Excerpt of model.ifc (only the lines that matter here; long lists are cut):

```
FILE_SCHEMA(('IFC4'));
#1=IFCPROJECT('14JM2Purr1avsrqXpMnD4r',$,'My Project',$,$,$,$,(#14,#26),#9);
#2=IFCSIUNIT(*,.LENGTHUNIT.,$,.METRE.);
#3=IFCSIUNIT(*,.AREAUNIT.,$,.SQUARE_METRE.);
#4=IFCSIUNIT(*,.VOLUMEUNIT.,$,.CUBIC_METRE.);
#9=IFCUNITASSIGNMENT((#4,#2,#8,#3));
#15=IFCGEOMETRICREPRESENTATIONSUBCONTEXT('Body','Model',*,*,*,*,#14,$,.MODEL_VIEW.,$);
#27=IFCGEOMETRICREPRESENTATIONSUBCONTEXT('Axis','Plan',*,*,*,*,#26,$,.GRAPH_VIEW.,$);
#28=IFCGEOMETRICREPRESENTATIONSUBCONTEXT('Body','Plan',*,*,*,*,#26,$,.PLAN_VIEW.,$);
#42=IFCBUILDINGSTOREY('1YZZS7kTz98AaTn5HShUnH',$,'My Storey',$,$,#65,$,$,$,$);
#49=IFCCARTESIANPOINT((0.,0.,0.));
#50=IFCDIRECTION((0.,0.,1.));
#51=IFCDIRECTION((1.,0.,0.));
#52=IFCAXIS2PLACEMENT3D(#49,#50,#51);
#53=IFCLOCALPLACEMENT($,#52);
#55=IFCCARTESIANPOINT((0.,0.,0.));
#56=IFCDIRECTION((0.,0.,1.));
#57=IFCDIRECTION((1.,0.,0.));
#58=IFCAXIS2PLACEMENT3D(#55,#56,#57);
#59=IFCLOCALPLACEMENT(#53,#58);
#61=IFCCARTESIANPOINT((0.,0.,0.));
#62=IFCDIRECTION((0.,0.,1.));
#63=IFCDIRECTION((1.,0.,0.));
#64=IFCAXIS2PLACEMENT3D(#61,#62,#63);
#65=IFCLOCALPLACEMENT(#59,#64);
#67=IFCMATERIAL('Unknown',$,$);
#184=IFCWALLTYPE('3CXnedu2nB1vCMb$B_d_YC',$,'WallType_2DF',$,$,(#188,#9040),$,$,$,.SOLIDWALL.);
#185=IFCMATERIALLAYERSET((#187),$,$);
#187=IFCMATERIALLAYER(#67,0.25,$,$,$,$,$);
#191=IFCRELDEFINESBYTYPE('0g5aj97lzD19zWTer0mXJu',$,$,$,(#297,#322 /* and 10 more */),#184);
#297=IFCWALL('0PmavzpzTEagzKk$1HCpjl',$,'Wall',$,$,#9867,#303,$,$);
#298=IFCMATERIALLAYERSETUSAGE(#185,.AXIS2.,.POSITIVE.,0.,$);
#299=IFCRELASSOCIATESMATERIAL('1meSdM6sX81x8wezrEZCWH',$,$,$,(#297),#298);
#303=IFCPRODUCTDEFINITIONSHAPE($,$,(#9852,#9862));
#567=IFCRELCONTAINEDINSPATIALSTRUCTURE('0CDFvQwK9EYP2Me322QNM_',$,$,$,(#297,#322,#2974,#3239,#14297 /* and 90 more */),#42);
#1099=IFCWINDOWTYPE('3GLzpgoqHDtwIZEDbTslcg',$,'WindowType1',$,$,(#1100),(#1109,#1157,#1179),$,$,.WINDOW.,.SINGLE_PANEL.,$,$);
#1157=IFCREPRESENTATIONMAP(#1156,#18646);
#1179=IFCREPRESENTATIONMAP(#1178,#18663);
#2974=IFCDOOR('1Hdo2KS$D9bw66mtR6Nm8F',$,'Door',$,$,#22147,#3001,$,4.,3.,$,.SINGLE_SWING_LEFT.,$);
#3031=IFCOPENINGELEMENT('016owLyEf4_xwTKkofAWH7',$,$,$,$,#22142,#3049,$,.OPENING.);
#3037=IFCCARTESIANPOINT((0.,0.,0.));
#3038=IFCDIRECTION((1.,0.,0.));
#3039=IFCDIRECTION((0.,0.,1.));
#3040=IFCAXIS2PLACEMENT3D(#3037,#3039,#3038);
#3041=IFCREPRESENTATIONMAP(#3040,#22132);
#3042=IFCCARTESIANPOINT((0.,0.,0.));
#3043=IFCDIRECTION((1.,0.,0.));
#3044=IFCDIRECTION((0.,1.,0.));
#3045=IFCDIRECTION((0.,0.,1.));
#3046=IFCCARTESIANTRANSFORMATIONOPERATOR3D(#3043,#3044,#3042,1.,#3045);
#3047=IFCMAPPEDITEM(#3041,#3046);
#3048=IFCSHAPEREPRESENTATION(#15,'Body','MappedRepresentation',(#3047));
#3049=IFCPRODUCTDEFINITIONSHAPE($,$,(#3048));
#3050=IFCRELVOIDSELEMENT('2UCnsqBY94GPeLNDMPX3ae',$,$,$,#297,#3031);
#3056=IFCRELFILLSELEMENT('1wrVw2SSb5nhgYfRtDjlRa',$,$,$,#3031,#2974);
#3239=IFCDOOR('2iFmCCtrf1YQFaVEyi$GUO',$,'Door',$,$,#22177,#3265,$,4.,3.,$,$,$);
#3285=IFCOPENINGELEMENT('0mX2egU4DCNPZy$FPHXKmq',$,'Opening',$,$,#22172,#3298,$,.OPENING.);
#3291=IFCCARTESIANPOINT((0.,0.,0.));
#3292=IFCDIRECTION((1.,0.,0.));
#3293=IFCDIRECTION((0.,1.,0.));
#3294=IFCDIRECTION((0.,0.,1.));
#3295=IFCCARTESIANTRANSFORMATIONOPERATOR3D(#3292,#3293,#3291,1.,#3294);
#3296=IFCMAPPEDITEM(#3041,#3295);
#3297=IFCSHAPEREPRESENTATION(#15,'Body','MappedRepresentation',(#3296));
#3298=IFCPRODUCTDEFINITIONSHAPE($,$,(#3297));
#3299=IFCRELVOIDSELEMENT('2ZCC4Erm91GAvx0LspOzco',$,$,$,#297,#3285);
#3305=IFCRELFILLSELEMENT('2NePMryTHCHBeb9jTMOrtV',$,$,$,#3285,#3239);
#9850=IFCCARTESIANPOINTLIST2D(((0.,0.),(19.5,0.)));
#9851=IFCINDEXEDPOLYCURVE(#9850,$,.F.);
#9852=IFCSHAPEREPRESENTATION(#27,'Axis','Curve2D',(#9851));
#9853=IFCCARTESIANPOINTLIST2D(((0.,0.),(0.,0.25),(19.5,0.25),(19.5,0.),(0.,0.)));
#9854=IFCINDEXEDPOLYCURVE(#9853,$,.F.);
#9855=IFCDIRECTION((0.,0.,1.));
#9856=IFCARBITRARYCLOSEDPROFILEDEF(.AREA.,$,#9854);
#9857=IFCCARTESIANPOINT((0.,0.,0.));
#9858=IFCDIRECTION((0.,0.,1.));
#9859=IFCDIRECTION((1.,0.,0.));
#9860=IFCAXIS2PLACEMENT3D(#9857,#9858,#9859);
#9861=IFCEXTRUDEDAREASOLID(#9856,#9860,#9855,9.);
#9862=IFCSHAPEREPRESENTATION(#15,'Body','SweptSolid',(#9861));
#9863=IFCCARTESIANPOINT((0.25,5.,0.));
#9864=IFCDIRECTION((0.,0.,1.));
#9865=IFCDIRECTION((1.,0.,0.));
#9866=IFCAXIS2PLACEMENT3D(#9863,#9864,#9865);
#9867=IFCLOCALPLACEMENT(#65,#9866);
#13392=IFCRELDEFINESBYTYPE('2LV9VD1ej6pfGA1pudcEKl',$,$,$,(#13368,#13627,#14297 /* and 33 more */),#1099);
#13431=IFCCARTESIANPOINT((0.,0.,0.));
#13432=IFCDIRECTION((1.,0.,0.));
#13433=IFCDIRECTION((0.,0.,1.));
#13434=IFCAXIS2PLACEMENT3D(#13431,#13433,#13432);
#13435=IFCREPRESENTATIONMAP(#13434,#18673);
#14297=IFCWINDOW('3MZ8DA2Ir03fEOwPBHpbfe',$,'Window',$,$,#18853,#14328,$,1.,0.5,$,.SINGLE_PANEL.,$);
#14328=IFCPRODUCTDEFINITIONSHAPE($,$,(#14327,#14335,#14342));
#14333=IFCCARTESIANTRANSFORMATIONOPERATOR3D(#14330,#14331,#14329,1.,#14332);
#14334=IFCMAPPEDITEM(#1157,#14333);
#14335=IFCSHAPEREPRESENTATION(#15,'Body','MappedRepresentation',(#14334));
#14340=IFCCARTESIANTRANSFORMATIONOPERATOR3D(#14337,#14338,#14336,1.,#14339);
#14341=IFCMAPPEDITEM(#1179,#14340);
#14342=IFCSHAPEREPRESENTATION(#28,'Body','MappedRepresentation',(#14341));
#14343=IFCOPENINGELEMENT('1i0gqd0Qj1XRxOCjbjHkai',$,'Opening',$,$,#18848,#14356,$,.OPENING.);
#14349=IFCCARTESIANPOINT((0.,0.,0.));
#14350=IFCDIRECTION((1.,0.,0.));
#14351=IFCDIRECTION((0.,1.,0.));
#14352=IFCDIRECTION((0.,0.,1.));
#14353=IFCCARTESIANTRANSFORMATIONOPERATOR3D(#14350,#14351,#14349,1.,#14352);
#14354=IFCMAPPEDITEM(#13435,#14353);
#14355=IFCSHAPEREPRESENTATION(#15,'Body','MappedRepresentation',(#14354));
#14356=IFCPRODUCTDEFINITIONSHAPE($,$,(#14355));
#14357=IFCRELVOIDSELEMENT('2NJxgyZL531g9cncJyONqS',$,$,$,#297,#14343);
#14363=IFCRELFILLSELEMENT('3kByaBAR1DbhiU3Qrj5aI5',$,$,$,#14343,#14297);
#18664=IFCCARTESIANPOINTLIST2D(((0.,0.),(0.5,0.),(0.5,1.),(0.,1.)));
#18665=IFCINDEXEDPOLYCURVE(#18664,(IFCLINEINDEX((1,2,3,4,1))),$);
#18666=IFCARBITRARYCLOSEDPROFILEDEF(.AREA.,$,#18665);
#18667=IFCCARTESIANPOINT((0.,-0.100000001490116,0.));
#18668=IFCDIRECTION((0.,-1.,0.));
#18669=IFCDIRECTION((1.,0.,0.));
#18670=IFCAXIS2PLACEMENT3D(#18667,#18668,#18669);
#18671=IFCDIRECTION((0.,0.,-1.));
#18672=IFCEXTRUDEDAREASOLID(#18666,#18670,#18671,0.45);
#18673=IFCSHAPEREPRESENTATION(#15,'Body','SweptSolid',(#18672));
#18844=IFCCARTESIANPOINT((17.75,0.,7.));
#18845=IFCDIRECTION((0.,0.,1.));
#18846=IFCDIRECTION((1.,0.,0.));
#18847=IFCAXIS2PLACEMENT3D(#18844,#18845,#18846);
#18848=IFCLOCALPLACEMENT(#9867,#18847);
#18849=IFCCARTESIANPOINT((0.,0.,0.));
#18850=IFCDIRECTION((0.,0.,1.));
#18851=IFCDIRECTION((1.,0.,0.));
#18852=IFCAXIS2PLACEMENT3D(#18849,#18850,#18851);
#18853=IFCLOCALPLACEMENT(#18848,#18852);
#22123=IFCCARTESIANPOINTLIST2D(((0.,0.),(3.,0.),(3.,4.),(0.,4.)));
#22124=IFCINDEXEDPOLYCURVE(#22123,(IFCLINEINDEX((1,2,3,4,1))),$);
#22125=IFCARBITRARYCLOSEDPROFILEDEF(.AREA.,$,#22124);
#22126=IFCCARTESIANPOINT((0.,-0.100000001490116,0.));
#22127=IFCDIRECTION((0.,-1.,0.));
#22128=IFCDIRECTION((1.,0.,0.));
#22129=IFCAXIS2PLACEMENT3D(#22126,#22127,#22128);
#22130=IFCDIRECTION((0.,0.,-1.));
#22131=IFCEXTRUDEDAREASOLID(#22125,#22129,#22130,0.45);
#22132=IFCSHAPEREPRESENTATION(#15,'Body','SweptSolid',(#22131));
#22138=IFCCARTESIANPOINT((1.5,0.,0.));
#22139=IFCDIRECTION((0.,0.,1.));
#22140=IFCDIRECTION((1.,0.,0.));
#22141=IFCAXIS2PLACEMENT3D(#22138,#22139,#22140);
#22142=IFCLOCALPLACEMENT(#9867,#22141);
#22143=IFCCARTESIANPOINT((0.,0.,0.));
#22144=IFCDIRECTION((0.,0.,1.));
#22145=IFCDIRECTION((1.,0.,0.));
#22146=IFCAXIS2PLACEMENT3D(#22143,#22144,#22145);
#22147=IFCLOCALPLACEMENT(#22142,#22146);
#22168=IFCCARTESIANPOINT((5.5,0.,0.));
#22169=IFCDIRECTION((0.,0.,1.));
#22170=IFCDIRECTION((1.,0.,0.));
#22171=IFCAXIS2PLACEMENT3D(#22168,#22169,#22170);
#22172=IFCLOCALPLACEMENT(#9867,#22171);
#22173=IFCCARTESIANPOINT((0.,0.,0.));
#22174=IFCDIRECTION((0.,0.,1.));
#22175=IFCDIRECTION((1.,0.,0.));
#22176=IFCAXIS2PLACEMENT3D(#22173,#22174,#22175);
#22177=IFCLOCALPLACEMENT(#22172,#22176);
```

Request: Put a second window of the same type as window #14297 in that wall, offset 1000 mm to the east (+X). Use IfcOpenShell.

```python
import ifcopenshell
import ifcopenshell.api.feature
import ifcopenshell.api.geometry
import ifcopenshell.api.root
import ifcopenshell.geom
import ifcopenshell.util.element
import ifcopenshell.util.placement
import ifcopenshell.util.shape

model = ifcopenshell.open("model.ifc")
settings = ifcopenshell.geom.settings()


def volume(element):
    """Net volume in cubic metres, openings subtracted."""
    shape = ifcopenshell.geom.create_shape(settings, element)
    return ifcopenshell.util.shape.get_volume(shape.geometry)


window = model.by_guid("3MZ8DA2Ir03fEOwPBHpbfe")
opening = window.FillsVoids[0].RelatingOpeningElement
wall = opening.VoidsElements[0].RelatingBuildingElement
before = volume(wall)
shift = ifcopenshell.util.placement.get_local_placement(wall.ObjectPlacement)[:3, 0] * 1.0

# copy_class copies the void relationship, type, container and properties, but no geometry.
new_opening = ifcopenshell.api.root.copy_class(model, product=opening)
new_opening.Representation = ifcopenshell.util.element.copy_deep(
    model, opening.Representation, exclude=["IfcGeometricRepresentationContext", "IfcRepresentationMap"]
)
new_window = ifcopenshell.api.root.copy_class(model, product=window)
new_window.Representation = ifcopenshell.util.element.copy_deep(
    model, window.Representation, exclude=["IfcGeometricRepresentationContext", "IfcRepresentationMap"]
)
ifcopenshell.api.feature.add_filling(model, opening=new_opening, element=new_window)

for old, new in ((opening, new_opening), (window, new_window)):
    matrix = ifcopenshell.util.placement.get_local_placement(old.ObjectPlacement)
    matrix[:3, 3] += shift
    ifcopenshell.api.geometry.edit_object_placement(model, product=new, matrix=matrix, is_si=False)

after = volume(wall)

print(f"wall volume {before:.3f} -> {after:.3f} m3")

model.write("model_edited.ifc")
```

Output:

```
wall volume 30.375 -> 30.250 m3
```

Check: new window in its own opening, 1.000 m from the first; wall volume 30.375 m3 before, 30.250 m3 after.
